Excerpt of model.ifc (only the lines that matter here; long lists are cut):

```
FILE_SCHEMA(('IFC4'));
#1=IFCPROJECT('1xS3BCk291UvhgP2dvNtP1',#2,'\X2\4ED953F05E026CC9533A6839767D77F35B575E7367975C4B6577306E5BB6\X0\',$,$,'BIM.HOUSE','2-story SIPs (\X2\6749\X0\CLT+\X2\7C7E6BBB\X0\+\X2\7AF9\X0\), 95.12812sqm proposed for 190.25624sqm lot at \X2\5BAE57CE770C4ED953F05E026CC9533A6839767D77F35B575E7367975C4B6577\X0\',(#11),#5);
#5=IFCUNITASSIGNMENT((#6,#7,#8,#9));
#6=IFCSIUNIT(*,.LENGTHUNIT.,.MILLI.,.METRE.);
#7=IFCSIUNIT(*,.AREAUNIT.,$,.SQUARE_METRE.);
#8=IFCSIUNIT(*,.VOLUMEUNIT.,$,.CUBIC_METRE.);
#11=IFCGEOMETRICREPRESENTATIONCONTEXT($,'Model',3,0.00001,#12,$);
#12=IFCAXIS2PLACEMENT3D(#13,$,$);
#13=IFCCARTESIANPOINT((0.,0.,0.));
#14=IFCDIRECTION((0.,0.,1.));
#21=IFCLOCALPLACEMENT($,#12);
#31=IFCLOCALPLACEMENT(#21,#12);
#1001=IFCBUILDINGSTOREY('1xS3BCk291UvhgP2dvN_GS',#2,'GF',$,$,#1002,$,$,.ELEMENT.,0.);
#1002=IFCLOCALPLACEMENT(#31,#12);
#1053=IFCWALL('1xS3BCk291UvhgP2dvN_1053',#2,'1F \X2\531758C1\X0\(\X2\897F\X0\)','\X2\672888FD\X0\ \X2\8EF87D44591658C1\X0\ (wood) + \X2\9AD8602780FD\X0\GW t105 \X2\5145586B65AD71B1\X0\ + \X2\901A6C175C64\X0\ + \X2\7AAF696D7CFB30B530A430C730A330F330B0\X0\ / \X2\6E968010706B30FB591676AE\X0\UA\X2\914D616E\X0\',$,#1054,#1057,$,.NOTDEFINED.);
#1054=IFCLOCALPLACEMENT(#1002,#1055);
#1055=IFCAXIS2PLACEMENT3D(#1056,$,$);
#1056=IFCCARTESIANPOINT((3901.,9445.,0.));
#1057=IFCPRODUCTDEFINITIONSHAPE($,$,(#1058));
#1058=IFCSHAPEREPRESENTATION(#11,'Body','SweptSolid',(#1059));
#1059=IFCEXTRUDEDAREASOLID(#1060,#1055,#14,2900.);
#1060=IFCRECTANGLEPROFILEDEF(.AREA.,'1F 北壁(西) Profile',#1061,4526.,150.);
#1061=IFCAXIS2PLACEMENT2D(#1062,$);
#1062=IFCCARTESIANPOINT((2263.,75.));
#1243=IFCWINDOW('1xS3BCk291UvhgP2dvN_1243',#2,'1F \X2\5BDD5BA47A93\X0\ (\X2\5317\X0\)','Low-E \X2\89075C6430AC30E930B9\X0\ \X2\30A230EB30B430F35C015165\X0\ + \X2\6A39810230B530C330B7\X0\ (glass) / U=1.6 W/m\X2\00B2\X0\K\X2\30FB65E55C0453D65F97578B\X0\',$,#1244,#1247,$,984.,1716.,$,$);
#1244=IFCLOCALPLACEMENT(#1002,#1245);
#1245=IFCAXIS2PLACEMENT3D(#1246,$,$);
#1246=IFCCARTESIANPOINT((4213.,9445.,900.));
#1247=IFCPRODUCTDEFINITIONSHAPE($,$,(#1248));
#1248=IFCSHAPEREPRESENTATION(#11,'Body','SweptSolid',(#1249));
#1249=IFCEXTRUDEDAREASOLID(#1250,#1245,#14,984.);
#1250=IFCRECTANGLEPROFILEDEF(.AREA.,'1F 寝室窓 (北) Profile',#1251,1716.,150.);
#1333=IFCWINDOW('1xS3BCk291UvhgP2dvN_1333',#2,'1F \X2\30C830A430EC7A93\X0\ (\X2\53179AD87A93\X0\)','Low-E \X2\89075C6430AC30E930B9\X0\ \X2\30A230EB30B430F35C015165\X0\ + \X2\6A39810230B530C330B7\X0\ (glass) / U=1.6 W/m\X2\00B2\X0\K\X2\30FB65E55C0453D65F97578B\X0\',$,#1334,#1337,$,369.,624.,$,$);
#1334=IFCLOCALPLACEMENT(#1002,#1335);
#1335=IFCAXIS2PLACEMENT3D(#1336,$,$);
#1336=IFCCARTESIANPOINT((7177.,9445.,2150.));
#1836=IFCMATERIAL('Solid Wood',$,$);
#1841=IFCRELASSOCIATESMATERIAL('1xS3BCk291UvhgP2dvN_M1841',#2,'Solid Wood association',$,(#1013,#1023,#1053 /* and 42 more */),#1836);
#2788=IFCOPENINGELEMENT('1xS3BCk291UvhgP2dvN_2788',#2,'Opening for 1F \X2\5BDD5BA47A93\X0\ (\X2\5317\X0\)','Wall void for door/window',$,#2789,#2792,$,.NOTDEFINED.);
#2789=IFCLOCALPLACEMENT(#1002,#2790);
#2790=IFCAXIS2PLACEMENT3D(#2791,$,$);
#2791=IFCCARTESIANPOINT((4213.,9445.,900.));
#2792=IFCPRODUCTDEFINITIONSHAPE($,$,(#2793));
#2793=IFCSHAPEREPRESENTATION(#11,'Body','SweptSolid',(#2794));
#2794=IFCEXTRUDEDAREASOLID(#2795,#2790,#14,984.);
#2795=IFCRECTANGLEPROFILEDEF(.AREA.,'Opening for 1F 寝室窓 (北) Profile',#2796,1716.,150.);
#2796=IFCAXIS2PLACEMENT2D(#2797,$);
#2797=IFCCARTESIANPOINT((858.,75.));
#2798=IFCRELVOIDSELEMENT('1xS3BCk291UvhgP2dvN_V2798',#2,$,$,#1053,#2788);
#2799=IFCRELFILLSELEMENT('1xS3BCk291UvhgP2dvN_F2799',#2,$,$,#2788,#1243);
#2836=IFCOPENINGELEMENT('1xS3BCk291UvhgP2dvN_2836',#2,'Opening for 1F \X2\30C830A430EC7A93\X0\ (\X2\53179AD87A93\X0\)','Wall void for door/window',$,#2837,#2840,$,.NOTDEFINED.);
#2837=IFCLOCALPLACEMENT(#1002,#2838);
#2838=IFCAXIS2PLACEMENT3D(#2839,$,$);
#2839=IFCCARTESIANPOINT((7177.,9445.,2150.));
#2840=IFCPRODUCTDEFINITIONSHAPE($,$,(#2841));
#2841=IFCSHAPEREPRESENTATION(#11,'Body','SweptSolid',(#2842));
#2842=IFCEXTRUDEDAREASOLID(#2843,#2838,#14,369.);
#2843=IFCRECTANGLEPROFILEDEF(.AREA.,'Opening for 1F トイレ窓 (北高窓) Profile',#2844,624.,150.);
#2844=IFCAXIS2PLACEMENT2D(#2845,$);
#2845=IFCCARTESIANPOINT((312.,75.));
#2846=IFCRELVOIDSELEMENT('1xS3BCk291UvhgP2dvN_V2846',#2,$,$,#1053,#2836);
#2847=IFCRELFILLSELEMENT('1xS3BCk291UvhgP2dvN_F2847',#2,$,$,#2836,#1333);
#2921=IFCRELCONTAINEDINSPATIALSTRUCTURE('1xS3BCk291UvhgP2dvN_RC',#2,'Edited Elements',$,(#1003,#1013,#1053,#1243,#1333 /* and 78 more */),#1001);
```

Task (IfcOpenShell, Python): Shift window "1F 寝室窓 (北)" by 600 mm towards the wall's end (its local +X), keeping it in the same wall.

```python
import ifcopenshell
import ifcopenshell.api.geometry
import ifcopenshell.util.placement

model = ifcopenshell.open("model.ifc")

window = model.by_id(1243)
opening = window.FillsVoids[0].RelatingOpeningElement
wall = opening.VoidsElements[0].RelatingBuildingElement

wall_matrix = ifcopenshell.util.placement.get_local_placement(wall.ObjectPlacement)
shift = wall_matrix[:3, 0] * 600.0
before = ifcopenshell.util.placement.get_local_placement(window.ObjectPlacement)[:3, 3].copy()

# The window is not placed relative to its opening, so move both.
for product in (opening, window):
    matrix = ifcopenshell.util.placement.get_local_placement(product.ObjectPlacement)
    matrix[:3, 3] += shift
    ifcopenshell.api.geometry.edit_object_placement(model, product=product, matrix=matrix, is_si=False)

after = ifcopenshell.util.placement.get_local_placement(window.ObjectPlacement)[:3, 3]
print("window moved by", (after - before).round(3) + 0.0)

model.write("model-out.ifc")
```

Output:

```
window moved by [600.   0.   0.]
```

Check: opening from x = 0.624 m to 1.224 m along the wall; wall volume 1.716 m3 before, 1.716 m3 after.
